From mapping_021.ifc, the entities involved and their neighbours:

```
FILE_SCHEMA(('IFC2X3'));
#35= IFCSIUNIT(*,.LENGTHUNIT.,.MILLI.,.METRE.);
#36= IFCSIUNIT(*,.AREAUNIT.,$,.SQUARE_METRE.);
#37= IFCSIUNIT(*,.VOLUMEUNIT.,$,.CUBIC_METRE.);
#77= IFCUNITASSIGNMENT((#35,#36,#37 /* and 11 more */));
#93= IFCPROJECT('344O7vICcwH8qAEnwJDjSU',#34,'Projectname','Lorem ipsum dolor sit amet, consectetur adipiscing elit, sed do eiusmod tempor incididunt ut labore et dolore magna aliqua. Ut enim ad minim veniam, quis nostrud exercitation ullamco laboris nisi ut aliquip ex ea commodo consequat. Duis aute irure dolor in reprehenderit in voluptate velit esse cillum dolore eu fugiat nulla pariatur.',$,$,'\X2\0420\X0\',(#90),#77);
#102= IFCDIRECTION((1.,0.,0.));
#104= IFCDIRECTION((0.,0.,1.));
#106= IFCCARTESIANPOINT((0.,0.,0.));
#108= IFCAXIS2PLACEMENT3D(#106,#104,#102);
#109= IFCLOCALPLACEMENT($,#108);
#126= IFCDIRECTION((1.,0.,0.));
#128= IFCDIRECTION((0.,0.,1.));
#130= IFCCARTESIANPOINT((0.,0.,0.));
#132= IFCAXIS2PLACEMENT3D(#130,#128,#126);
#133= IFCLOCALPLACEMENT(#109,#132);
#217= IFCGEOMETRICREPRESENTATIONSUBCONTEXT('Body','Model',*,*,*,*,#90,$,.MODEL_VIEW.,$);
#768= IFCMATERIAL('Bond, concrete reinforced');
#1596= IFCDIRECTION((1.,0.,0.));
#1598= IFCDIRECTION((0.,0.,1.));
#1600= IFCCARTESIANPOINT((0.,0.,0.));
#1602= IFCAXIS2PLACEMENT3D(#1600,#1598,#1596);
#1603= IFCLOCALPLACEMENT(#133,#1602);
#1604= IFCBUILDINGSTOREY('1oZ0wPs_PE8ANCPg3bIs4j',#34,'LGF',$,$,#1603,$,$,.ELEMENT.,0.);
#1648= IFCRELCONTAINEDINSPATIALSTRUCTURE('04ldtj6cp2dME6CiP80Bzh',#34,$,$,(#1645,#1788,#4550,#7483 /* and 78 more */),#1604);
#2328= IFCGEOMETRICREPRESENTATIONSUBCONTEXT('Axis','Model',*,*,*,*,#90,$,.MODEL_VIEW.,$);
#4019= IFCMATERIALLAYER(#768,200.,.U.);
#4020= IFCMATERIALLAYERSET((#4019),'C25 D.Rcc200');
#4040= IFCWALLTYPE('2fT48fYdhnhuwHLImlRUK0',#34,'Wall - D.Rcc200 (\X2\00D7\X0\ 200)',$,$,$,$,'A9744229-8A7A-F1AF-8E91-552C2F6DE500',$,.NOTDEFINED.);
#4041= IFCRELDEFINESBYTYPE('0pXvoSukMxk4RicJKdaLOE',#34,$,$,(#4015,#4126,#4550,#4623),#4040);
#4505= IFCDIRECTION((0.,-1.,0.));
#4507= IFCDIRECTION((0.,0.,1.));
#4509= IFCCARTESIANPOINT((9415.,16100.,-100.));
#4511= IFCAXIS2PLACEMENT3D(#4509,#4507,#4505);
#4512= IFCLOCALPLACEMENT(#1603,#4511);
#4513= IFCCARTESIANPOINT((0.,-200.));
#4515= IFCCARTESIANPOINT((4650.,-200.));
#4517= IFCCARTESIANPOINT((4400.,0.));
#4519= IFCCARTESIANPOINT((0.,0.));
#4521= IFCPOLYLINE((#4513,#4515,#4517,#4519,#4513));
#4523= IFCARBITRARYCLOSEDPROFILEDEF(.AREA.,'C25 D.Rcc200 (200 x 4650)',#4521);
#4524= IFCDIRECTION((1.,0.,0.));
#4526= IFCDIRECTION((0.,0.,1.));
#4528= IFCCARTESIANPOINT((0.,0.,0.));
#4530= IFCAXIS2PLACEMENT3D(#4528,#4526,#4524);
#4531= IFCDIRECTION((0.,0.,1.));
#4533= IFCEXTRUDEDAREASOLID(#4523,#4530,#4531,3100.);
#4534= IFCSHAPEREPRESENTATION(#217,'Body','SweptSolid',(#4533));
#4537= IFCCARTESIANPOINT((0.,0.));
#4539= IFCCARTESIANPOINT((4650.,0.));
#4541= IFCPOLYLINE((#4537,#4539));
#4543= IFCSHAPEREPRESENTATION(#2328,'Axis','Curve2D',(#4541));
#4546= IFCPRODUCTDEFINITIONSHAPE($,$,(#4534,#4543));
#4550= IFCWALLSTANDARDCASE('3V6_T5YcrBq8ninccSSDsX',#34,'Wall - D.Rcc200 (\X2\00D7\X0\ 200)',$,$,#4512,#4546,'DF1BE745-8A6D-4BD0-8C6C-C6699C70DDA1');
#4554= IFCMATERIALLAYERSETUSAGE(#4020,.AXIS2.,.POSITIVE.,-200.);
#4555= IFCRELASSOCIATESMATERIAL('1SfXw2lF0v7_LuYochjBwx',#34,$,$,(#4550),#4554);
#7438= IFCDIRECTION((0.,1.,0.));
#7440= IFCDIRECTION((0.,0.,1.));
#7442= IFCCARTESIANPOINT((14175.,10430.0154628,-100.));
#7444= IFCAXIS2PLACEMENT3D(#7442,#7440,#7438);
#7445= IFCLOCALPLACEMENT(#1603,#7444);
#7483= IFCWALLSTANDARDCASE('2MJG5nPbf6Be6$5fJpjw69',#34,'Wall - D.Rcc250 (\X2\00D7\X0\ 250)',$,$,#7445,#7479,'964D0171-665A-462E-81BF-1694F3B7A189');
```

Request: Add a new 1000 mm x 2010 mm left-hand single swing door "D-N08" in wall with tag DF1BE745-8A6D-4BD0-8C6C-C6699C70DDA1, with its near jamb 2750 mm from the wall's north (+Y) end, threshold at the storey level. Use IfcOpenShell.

```python
import numpy as np
import ifcopenshell
import ifcopenshell.api.feature
import ifcopenshell.api.geometry
import ifcopenshell.api.root
import ifcopenshell.api.spatial
import ifcopenshell.api.type
import ifcopenshell.geom
import ifcopenshell.util.element
import ifcopenshell.util.placement
import ifcopenshell.util.representation
import ifcopenshell.util.shape
import ifcopenshell.util.unit

model = ifcopenshell.open("mapping_021.ifc")
unit_scale = ifcopenshell.util.unit.calculate_unit_scale(model)
settings = ifcopenshell.geom.settings()


def volume(element):
    """Net volume in cubic metres, openings subtracted."""
    shape = ifcopenshell.geom.create_shape(settings, element)
    return ifcopenshell.util.shape.get_volume(shape.geometry)


wall = model.by_guid("3V6_T5YcrBq8ninccSSDsX")
storey = ifcopenshell.util.element.get_container(wall, ifc_class="IfcBuildingStorey")
context = ifcopenshell.util.representation.get_context(model, "Model", "Body", "MODEL_VIEW")
before = volume(wall)

width, height, from_end, sill = 1, 2.01, 2.75, 0.0  # metres

# The wall runs along its own X axis, and the end named is its -X end.
wall_shape = ifcopenshell.geom.create_shape(settings, wall)
x, y, z = ifcopenshell.util.shape.get_vertices(wall_shape.geometry).T
start = x.min() + from_end
face, thickness = float(y.min()), float(y.max() - y.min())
wall_matrix = ifcopenshell.util.placement.get_local_placement(wall.ObjectPlacement)
level = ifcopenshell.util.placement.get_local_placement(storey.ObjectPlacement)[2, 3]


def in_wall(x, y):
    """Placement at x, y metres in the wall's axes, at sill height."""
    matrix = wall_matrix.copy()
    matrix[:, 3] = wall_matrix @ np.array([x / unit_scale, y / unit_scale, 0.0, 1.0])
    matrix[2, 3] = level + sill / unit_scale
    return matrix


# Opening: a box that overshoots both wall faces by 50 mm.
opening = ifcopenshell.api.root.create_entity(model, ifc_class="IfcOpeningElement")
box = ifcopenshell.api.geometry.add_wall_representation(
    model, context=context, length=width, height=height, thickness=thickness + 0.1
)
ifcopenshell.api.geometry.assign_representation(model, product=opening, representation=box)
ifcopenshell.api.geometry.edit_object_placement(model, product=opening, matrix=in_wall(start, face - 0.05), is_si=False)
ifcopenshell.api.feature.add_feature(model, feature=opening, element=wall)

door = ifcopenshell.api.root.create_entity(model, ifc_class="IfcDoor", name="D-N08")
door.OverallWidth, door.OverallHeight = width / unit_scale, height / unit_scale
body = ifcopenshell.api.geometry.add_door_representation(
    model,
    context=context,
    overall_width=door.OverallWidth,
    overall_height=door.OverallHeight,
    operation_type="SINGLE_SWING_LEFT",
    lining_properties={"LiningDepth": thickness / unit_scale, "ThresholdDepth": thickness / unit_scale},
)
ifcopenshell.api.geometry.assign_representation(model, product=door, representation=body)
ifcopenshell.api.spatial.assign_container(model, products=[door], relating_structure=storey)
fills = ifcopenshell.api.feature.add_filling(model, opening=opening, element=door)
fills.OwnerHistory = door.OwnerHistory  # required in IFC2X3

# IFC2X3 keeps the operation on the door style.
style = ifcopenshell.api.root.create_entity(model, ifc_class="IfcDoorStyle", name="D-N08")
style.OperationType, style.ConstructionType = "SINGLE_SWING_LEFT", "NOTDEFINED"
style.ParameterTakesPrecedence = style.Sizeable = False
ifcopenshell.api.type.assign_type(model, related_objects=[door], relating_type=style)

# The lining spans the wall, so the door starts at the wall face.
ifcopenshell.api.geometry.edit_object_placement(model, product=door, matrix=in_wall(start, face), is_si=False)

after = volume(wall)

print(f"wall volume {before:.3f} -> {after:.3f} m3")

model.write("mapping_021-out.ifc")
```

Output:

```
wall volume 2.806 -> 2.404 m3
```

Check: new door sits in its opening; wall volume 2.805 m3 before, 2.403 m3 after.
